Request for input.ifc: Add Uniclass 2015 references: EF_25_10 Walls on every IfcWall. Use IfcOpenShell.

First a look at what the model holds.

```python
import ifcopenshell

model = ifcopenshell.open("input.ifc")
print(model.schema)
print("classifications:", [c.Name for c in model.by_type("IfcClassification")])
for ifc_class in ("IfcDoor", "IfcRoof", "IfcStair", "IfcWall", "IfcWindow"):
    print(ifc_class, len(model.by_type(ifc_class)))
```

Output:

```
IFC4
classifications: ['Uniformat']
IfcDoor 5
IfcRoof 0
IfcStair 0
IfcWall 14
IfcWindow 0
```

```python
import ifcopenshell
import ifcopenshell.api.classification

model = ifcopenshell.open("input.ifc")

system = ifcopenshell.api.classification.add_classification(model, classification="Uniclass 2015")

codes = {
    "IfcWall": ("EF_25_10", "Walls"),
}
for ifc_class, (code, name) in codes.items():
    products = model.by_type(ifc_class)
    ifcopenshell.api.classification.add_reference(
        model, products=products, classification=system, identification=code, name=name
    )
    print(code, len(products))

model.write("input_updated.ifc")
```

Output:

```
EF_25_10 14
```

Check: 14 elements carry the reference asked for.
